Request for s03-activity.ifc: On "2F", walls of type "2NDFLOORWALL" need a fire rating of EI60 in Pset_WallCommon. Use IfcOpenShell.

First a look at what the model holds.

```python
import ifcopenshell
import ifcopenshell.util.element

model = ifcopenshell.open("s03-activity.ifc")
print(model.schema)
storey = next(s for s in model.by_type("IfcBuildingStorey") if s.Name == "2F")
walls = [e for e in ifcopenshell.util.element.get_decomposition(storey) if e.is_a("IfcWall")]
seen = {}
for e in walls:
    element_type = ifcopenshell.util.element.get_type(e)
    key = (element_type.Name if element_type != e and element_type else None, ifcopenshell.util.element.get_pset(e, "Pset_WallCommon", "FireRating"))
    seen[key] = seen.get(key, 0) + 1
for (name, value), count in sorted(seen.items(), key=str):
    print(count, "x", name, "|", value)
```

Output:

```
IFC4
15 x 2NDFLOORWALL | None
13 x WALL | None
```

```python
import ifcopenshell
import ifcopenshell.api.pset
import ifcopenshell.util.element

model = ifcopenshell.open("s03-activity.ifc")

storey = next(s for s in model.by_type("IfcBuildingStorey") if s.Name == "2F")
walls = [e for e in ifcopenshell.util.element.get_decomposition(storey) if e.is_a("IfcWall")]

count = 0
for e in walls:
    element_type = ifcopenshell.util.element.get_type(e)
    if element_type in (None, e) or element_type.Name != "2NDFLOORWALL":
        continue
    # add_pset returns the element's existing set when there is one.
    pset = ifcopenshell.api.pset.add_pset(model, product=e, name="Pset_WallCommon")
    ifcopenshell.api.pset.edit_pset(model, pset=pset, properties={"FireRating": "EI60"})
    count += 1

print(count, "walls updated")

model.write("s03-activity_edited.ifc")
```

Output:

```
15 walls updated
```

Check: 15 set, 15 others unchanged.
